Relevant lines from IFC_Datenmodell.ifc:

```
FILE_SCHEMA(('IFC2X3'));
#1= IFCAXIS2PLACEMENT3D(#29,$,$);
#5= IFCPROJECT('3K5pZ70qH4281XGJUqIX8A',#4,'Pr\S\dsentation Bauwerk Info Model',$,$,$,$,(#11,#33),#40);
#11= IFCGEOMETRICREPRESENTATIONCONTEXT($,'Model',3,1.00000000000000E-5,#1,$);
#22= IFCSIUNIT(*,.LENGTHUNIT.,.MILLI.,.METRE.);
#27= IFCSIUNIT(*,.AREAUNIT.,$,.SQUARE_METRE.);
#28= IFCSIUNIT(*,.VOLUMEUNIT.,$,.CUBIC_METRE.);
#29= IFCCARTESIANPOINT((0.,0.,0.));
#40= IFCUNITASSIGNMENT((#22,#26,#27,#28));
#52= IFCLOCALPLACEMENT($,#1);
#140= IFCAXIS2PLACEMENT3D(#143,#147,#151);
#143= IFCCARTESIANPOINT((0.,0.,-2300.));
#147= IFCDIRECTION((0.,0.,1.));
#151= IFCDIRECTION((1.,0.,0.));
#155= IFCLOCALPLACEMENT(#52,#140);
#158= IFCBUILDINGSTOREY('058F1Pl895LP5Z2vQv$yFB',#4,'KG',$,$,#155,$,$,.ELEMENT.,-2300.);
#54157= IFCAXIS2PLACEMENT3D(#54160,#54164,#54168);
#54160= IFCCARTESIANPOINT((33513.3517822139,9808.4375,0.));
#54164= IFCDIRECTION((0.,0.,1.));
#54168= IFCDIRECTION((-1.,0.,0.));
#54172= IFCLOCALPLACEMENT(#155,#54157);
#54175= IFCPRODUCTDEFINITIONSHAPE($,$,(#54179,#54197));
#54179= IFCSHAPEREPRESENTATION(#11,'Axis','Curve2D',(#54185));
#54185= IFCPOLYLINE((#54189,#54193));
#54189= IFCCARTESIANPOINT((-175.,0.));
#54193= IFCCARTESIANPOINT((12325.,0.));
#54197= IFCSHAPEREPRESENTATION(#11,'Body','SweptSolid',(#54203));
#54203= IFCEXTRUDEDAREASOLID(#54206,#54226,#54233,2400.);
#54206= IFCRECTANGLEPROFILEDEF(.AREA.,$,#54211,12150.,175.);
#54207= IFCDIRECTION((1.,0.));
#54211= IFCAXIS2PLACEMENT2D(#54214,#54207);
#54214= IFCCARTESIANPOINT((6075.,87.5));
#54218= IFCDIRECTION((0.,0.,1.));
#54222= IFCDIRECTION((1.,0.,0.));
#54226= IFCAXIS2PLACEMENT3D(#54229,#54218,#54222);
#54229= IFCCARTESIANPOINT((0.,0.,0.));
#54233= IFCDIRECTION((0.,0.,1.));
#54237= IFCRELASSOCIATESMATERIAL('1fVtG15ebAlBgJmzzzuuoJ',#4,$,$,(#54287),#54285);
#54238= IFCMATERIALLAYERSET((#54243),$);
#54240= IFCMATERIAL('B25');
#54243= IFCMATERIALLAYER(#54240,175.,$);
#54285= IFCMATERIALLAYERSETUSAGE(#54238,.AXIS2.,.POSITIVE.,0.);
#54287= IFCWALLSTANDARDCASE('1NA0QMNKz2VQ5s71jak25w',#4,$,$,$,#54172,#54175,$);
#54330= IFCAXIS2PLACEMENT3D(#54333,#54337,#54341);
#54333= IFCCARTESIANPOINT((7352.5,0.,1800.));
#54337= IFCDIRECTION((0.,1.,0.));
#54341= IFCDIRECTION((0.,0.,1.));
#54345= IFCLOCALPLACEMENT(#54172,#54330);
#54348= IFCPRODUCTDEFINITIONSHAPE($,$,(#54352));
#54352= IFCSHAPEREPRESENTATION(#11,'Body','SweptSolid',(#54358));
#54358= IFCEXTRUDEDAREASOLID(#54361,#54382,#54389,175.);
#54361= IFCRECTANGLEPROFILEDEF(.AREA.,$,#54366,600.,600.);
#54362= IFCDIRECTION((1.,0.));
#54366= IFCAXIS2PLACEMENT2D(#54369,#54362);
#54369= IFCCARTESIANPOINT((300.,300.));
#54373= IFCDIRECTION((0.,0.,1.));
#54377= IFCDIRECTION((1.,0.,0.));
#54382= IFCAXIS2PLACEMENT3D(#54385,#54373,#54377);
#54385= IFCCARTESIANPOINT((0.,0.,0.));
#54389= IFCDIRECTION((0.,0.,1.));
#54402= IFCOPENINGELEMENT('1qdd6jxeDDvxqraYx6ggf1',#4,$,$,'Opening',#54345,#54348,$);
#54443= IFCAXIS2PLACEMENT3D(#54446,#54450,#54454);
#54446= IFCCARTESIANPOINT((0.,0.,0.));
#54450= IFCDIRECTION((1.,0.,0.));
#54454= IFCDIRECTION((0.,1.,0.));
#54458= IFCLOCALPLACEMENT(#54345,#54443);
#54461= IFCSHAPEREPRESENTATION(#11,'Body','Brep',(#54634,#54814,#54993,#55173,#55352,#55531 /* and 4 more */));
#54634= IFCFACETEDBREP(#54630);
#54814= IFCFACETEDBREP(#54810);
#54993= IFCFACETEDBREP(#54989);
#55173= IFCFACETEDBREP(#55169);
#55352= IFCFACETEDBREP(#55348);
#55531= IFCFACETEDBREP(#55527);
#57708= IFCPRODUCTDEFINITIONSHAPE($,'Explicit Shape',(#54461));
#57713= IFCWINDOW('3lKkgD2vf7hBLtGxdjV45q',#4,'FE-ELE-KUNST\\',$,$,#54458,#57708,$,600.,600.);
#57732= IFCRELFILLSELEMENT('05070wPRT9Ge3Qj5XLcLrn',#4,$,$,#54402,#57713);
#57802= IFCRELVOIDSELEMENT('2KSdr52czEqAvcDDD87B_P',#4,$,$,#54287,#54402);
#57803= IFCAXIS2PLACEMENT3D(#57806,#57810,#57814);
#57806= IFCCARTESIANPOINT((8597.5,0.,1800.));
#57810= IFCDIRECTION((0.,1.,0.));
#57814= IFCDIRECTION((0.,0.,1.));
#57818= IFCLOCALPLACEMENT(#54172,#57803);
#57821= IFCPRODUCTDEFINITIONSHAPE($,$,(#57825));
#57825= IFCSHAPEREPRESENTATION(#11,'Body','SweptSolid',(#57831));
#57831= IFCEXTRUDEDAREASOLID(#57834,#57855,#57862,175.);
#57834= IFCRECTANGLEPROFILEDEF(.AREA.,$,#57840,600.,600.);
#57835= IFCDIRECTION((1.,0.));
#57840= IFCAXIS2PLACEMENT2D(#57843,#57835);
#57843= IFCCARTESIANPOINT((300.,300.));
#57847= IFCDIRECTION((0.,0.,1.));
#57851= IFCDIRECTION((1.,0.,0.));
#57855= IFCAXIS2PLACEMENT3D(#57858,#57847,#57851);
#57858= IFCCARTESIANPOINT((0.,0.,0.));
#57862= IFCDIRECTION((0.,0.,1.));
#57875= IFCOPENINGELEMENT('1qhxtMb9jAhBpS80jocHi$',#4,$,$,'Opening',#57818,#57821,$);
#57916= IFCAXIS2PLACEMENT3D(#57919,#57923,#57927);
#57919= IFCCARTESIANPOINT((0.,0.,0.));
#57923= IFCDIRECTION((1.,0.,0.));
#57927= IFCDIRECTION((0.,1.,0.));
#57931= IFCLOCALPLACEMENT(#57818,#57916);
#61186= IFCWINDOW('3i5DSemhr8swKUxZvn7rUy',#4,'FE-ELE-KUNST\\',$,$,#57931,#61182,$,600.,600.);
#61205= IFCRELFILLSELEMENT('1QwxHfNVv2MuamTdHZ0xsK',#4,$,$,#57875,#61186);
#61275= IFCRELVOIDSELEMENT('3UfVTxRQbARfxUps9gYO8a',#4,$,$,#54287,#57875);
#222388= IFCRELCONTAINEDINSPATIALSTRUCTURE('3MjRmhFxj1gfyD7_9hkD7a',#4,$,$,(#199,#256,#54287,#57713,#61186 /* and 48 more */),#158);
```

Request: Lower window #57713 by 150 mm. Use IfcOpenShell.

```python
import numpy as np
import ifcopenshell
import ifcopenshell.api.geometry
import ifcopenshell.util.placement
import ifcopenshell.util.unit

model = ifcopenshell.open("IFC_Datenmodell.ifc")
unit_scale = ifcopenshell.util.unit.calculate_unit_scale(model)

window = model.by_guid("3lKkgD2vf7hBLtGxdjV45q")
opening = window.FillsVoids[0].RelatingOpeningElement
dz = -150.0

shift = np.array([0.0, 0.0, dz])
# The window is placed relative to its opening, so it follows when the opening moves.
matrix = ifcopenshell.util.placement.get_local_placement(opening.ObjectPlacement)
matrix[:3, 3] += shift
ifcopenshell.api.geometry.edit_object_placement(
    model, product=opening, matrix=matrix, is_si=False, should_transform_children=True
)

print(f"moved by {dz * unit_scale:+.3f} m")

model.write("IFC_Datenmodell_rev.ifc")
```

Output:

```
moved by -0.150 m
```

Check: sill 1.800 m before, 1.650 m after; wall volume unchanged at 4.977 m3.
